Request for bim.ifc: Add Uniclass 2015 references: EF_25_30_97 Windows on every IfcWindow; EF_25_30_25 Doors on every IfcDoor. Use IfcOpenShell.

First a look at what the model holds.

```python
import ifcopenshell

model = ifcopenshell.open("bim.ifc")
print(model.schema)
print("classifications:", [c.Name for c in model.by_type("IfcClassification")])
for ifc_class in ("IfcDoor", "IfcRoof", "IfcStair", "IfcWall", "IfcWindow"):
    print(ifc_class, len(model.by_type(ifc_class)))
```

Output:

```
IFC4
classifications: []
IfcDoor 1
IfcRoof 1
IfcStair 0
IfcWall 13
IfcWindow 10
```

```python
import ifcopenshell
import ifcopenshell.api.classification

model = ifcopenshell.open("bim.ifc")

system = ifcopenshell.api.classification.add_classification(model, classification="Uniclass 2015")

codes = {
    "IfcWindow": ("EF_25_30_97", "Windows"),
    "IfcDoor": ("EF_25_30_25", "Doors"),
}
for ifc_class, (code, name) in codes.items():
    products = model.by_type(ifc_class)
    ifcopenshell.api.classification.add_reference(
        model, products=products, classification=system, identification=code, name=name
    )
    print(code, len(products))

model.write("bim_updated.ifc")
```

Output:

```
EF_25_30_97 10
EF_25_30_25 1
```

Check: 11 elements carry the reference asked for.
